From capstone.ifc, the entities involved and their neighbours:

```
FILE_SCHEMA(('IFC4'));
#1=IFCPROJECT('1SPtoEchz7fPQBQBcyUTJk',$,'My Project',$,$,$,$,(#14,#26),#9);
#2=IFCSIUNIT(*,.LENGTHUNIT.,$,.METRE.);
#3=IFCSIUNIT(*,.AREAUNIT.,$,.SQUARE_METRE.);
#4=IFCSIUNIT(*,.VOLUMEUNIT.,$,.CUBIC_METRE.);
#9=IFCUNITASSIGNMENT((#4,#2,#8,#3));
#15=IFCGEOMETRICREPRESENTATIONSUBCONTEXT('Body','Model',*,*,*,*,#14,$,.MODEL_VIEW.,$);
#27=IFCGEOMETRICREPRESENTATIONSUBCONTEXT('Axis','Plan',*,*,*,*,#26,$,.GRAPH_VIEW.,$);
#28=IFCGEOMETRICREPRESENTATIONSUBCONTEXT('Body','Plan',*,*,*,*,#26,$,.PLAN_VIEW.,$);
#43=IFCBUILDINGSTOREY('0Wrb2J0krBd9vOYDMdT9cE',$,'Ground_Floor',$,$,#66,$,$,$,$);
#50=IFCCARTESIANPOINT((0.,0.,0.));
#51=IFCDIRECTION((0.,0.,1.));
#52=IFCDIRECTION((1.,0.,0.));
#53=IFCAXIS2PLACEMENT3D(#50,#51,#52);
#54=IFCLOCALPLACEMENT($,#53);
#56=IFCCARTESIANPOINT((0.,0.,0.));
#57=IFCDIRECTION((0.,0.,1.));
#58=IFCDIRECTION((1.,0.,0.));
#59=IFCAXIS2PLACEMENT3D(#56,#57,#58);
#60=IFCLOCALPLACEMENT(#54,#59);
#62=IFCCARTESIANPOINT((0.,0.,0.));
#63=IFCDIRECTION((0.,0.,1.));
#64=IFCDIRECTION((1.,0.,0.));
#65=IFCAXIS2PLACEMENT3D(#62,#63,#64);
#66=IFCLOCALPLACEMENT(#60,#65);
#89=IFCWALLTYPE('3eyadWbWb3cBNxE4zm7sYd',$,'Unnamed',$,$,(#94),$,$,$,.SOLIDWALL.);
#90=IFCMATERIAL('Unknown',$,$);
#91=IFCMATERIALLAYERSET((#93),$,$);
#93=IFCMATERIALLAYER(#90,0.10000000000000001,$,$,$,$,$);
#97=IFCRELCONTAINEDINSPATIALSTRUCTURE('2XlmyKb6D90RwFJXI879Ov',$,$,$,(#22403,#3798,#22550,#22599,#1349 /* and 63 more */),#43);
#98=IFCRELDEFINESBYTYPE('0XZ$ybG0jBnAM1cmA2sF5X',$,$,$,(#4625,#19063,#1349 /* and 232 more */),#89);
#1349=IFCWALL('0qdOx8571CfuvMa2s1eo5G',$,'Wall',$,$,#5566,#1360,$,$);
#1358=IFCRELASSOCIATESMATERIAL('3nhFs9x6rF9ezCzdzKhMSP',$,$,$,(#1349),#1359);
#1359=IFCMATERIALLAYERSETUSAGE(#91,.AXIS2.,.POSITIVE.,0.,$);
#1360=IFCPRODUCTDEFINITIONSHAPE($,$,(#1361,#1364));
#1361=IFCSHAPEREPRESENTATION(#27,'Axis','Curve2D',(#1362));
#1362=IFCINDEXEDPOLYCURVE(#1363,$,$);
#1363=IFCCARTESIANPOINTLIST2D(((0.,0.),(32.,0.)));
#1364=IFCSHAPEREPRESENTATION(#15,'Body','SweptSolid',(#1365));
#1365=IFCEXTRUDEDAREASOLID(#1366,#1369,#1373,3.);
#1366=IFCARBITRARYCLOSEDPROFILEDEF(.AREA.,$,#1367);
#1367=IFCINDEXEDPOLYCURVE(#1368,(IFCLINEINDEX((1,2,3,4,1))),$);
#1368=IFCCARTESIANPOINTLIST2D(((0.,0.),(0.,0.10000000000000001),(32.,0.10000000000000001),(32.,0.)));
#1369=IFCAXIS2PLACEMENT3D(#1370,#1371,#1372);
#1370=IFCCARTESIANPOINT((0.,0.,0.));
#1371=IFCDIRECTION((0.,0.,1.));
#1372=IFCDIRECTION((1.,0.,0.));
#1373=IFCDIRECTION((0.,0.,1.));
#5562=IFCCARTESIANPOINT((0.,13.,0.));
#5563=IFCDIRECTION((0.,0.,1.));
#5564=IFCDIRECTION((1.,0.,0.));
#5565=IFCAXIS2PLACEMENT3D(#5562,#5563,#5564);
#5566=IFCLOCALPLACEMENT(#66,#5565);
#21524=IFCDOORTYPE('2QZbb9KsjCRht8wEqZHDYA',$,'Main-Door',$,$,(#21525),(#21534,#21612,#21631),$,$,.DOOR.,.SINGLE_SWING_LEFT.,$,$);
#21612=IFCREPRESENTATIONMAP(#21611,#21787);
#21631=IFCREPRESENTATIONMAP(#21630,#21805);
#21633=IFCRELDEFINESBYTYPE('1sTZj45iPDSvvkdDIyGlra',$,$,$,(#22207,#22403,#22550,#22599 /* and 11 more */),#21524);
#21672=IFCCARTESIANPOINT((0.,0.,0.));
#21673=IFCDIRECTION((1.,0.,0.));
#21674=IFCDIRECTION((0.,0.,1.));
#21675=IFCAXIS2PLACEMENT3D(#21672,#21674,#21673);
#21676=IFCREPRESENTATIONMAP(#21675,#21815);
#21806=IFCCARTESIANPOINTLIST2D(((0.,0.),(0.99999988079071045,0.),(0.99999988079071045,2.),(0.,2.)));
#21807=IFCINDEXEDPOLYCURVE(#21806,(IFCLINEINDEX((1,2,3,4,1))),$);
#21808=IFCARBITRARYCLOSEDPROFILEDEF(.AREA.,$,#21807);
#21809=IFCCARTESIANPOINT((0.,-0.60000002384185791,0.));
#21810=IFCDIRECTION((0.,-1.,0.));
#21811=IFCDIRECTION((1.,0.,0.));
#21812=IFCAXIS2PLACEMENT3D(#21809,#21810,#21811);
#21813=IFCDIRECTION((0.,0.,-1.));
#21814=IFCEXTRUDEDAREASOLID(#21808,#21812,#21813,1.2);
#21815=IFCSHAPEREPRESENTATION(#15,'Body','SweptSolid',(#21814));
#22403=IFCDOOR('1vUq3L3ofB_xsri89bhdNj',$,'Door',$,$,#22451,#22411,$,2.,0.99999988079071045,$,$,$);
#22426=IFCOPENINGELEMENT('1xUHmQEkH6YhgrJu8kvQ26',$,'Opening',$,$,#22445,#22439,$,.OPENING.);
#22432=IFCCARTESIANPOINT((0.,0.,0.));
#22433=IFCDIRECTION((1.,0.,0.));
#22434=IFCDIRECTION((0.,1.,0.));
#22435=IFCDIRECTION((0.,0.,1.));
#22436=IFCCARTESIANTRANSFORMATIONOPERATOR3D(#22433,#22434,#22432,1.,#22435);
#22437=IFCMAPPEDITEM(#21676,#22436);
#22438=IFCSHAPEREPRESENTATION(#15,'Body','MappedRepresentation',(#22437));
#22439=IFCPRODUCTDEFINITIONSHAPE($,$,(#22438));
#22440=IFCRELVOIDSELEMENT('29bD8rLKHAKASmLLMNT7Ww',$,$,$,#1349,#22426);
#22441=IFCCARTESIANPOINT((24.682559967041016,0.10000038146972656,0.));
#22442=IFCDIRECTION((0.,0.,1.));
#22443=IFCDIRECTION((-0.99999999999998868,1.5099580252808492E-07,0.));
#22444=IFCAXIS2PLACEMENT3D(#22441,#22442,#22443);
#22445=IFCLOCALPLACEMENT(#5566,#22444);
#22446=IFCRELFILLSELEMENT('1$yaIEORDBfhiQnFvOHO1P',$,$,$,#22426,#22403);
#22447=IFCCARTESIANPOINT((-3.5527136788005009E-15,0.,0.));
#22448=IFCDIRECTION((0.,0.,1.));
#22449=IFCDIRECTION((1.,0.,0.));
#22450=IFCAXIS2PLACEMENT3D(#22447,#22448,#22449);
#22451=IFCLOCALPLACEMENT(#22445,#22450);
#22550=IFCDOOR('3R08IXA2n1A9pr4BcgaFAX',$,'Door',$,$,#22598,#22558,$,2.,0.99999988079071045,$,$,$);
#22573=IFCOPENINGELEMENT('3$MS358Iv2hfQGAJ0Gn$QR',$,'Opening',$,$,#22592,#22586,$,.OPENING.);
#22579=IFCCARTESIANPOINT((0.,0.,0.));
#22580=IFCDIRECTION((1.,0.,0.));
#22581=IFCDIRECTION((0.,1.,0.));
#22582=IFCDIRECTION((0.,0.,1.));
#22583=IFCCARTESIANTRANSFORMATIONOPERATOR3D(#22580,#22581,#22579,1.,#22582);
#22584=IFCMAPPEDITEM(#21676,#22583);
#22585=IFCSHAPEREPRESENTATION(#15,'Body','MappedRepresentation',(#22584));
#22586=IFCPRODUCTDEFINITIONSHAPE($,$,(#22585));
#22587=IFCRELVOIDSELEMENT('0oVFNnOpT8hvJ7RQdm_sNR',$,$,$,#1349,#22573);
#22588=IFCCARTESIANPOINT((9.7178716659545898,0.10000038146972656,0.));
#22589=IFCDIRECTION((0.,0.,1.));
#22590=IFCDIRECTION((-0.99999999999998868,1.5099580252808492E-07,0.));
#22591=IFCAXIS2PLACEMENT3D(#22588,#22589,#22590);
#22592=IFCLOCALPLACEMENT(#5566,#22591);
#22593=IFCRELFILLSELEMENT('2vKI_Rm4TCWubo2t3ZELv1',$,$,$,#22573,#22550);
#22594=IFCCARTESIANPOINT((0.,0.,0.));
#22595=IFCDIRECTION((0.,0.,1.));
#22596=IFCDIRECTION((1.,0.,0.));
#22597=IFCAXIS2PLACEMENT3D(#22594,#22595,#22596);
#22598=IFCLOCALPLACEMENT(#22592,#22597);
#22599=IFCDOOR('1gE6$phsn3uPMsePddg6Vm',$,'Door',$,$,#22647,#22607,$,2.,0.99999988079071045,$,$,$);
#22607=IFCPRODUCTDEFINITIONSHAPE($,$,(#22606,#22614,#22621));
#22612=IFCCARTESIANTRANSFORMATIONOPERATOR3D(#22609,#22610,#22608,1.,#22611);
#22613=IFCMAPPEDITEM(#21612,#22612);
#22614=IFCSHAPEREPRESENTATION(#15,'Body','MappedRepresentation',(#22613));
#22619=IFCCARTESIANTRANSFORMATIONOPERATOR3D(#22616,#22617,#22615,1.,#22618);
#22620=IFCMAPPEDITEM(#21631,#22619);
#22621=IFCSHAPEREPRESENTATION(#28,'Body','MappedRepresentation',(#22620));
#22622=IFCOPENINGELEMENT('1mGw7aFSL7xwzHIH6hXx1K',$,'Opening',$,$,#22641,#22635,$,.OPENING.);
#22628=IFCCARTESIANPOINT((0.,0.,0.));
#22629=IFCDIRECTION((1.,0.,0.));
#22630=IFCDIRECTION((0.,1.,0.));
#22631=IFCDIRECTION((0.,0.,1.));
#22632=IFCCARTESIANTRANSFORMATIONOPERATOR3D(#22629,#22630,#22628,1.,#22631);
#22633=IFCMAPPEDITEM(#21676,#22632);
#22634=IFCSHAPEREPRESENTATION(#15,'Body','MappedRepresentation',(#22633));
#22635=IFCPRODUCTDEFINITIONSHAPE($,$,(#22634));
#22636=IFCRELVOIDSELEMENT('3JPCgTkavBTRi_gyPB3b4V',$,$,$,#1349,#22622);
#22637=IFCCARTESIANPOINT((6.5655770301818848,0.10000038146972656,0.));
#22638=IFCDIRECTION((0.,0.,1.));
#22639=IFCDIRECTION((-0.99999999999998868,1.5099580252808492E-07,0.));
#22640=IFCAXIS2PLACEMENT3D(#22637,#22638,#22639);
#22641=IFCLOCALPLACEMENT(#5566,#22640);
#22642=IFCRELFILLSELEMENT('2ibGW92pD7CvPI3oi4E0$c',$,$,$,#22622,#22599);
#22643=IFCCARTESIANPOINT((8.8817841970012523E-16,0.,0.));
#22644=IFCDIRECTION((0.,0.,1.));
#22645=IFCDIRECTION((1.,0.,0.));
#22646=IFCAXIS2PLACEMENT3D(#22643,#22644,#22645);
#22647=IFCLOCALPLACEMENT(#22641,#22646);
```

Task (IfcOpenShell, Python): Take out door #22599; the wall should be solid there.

```python
import ifcopenshell
import ifcopenshell.api.feature
import ifcopenshell.api.root
import ifcopenshell.geom
import ifcopenshell.util.shape

model = ifcopenshell.open("capstone.ifc")
settings = ifcopenshell.geom.settings()


def volume(element):
    """Net volume in cubic metres, openings subtracted."""
    shape = ifcopenshell.geom.create_shape(settings, element)
    return ifcopenshell.util.shape.get_volume(shape.geometry)


door = model.by_guid("1gE6$phsn3uPMsePddg6Vm")
opening = door.FillsVoids[0].RelatingOpeningElement
wall = opening.VoidsElements[0].RelatingBuildingElement
before = volume(wall)

ifcopenshell.api.root.remove_product(model, product=door)
ifcopenshell.api.feature.remove_feature(model, feature=opening)

after = volume(wall)

print(f"wall volume {before:.3f} -> {after:.3f} m3")

model.write("capstone_updated.ifc")
```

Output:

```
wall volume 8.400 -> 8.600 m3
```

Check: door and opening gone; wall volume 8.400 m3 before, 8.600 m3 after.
